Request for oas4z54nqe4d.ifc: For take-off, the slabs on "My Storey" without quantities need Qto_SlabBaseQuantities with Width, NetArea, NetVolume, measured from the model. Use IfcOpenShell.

First a look at what the model holds.

```python
import ifcopenshell
import ifcopenshell.util.element
import ifcopenshell.util.unit

model = ifcopenshell.open("oas4z54nqe4d.ifc")
print(model.schema)
for unit_type in ("LENGTHUNIT", "AREAUNIT", "VOLUMEUNIT"):
    print(unit_type, ifcopenshell.util.unit.calculate_unit_scale(model, unit_type))
storey = next(s for s in model.by_type("IfcBuildingStorey") if s.Name == "My Storey")
slabs = [e for e in ifcopenshell.util.element.get_decomposition(storey) if e.is_a("IfcSlab")]
for e in sorted(slabs, key=lambda e: e.id()):
    print(e.id(), e.is_a(), e.Name, list(ifcopenshell.util.element.get_psets(e, qtos_only=True)), sep=" | ")
```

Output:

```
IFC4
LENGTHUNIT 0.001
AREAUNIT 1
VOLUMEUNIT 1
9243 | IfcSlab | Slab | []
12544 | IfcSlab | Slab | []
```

```python
import ifcopenshell
import ifcopenshell.api.pset
import ifcopenshell.geom
import ifcopenshell.util.element
import ifcopenshell.util.shape
import ifcopenshell.util.unit

model = ifcopenshell.open("oas4z54nqe4d.ifc")
unit_scale = ifcopenshell.util.unit.calculate_unit_scale(model)
area_scale = ifcopenshell.util.unit.calculate_unit_scale(model, "AREAUNIT")
volume_scale = ifcopenshell.util.unit.calculate_unit_scale(model, "VOLUMEUNIT")
settings = ifcopenshell.geom.settings()

storey = next(s for s in model.by_type("IfcBuildingStorey") if s.Name == "My Storey")
slabs = [e for e in ifcopenshell.util.element.get_decomposition(storey) if e.is_a("IfcSlab")]

for e in sorted(slabs, key=lambda e: e.id()):
    if ifcopenshell.util.element.get_psets(e, qtos_only=True, should_inherit=False):
        continue
    # Geometry comes back in metres, in the element's own axes.
    shape = ifcopenshell.geom.create_shape(settings, e)
    values = {
        "Width": ifcopenshell.util.shape.get_z(shape.geometry) / unit_scale,
        "NetArea": ifcopenshell.util.shape.get_footprint_area(shape.geometry) / area_scale,
        "NetVolume": ifcopenshell.util.shape.get_volume(shape.geometry) / volume_scale,
    }
    qto = ifcopenshell.api.pset.add_qto(model, product=e, name="Qto_SlabBaseQuantities")
    ifcopenshell.api.pset.edit_qto(model, qto=qto, properties=values)
    print(e.id(), {k: round(v, 3) for k, v in values.items()})

model.write("oas4z54nqe4d-out.ifc")
```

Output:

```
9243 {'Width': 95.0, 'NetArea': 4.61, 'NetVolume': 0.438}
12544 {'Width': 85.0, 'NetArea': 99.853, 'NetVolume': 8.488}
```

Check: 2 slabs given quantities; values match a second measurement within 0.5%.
